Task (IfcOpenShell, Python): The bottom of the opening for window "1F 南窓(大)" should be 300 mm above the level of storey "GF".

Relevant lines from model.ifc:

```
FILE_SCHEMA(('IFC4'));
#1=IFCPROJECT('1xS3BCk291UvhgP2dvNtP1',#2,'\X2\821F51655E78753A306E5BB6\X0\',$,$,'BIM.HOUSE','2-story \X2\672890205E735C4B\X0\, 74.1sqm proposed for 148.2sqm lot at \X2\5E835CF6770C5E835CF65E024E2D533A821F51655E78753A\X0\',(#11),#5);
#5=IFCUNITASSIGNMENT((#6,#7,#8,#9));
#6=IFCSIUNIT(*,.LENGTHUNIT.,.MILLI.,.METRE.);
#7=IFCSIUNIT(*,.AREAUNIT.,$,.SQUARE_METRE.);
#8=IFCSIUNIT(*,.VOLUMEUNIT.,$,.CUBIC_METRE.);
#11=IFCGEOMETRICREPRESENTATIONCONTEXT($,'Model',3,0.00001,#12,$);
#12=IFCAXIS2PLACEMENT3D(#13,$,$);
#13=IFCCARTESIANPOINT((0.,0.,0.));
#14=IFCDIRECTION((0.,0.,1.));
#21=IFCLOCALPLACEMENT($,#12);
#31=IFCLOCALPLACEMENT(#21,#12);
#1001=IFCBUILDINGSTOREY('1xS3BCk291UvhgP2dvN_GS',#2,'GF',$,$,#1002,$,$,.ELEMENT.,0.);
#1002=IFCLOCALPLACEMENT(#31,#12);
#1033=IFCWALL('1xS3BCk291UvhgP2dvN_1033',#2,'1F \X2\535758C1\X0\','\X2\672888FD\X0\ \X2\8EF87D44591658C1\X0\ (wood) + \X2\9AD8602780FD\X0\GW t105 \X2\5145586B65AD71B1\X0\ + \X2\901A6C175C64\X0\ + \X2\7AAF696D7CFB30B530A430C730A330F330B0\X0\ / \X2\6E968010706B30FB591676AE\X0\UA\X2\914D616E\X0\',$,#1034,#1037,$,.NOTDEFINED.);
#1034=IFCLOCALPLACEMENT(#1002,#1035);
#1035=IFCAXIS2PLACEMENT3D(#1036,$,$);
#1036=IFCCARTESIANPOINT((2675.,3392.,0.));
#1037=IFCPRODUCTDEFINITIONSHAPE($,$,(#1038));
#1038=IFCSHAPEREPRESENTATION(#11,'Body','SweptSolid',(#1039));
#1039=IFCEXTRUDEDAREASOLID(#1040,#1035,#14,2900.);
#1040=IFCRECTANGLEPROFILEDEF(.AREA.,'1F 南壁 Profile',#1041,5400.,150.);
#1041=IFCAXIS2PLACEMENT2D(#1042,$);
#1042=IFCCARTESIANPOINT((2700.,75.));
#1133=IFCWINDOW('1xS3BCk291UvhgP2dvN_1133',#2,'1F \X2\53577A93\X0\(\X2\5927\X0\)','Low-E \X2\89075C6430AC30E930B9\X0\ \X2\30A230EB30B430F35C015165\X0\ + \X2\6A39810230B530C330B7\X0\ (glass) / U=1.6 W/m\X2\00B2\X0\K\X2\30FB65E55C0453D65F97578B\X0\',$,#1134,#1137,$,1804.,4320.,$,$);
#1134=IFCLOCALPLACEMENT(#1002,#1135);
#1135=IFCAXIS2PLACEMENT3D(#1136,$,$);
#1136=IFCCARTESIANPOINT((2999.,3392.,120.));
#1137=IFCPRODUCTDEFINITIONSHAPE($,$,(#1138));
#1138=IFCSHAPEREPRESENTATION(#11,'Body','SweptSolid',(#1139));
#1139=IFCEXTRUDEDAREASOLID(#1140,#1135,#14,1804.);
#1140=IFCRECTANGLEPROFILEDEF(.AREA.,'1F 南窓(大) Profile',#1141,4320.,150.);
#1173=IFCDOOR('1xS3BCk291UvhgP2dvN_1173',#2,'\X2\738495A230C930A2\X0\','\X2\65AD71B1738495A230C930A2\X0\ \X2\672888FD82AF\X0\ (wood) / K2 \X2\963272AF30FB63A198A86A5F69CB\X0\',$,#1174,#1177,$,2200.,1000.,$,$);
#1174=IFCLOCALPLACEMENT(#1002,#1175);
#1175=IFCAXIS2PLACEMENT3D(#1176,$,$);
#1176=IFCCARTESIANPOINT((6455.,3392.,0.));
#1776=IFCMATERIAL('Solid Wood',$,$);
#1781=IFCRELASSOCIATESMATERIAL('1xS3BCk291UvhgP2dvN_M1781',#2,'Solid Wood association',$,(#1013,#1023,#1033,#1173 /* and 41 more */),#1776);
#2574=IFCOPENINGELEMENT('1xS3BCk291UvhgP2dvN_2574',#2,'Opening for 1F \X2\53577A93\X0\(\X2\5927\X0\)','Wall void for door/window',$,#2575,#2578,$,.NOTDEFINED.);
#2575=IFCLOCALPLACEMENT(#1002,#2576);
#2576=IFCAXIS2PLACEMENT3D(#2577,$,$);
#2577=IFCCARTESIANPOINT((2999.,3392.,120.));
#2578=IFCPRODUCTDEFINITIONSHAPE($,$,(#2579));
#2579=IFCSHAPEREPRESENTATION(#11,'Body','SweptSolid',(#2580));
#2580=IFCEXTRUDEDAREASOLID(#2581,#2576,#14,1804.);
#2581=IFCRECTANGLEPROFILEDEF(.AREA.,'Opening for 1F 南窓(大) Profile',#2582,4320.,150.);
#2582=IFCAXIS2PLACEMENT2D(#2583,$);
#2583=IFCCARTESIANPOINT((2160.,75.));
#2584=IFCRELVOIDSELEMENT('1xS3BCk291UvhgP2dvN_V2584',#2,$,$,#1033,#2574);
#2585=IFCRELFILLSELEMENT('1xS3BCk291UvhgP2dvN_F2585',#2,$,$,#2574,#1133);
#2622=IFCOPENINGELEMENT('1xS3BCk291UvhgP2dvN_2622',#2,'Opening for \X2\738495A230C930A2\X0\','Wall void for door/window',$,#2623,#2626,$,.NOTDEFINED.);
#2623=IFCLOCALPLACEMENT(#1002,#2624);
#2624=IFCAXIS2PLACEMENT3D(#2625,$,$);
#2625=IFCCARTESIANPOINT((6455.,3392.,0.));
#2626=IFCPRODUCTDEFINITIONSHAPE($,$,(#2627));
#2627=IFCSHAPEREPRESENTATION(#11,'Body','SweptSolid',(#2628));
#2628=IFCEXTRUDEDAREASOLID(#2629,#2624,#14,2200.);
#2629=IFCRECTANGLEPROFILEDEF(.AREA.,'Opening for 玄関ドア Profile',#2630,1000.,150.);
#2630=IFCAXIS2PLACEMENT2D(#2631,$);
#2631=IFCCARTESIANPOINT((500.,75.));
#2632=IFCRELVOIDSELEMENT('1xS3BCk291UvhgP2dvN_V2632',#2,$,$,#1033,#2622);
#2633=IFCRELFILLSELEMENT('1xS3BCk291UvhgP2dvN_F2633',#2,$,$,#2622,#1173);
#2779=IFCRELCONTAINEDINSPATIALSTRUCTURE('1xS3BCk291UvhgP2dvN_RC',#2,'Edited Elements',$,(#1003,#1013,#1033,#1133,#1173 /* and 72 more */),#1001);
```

```python
import numpy as np
import ifcopenshell
import ifcopenshell.api.geometry
import ifcopenshell.geom
import ifcopenshell.util.element
import ifcopenshell.util.placement
import ifcopenshell.util.shape
import ifcopenshell.util.unit

model = ifcopenshell.open("model.ifc")
unit_scale = ifcopenshell.util.unit.calculate_unit_scale(model)

window = model.by_guid("1xS3BCk291UvhgP2dvN_1133")
opening = window.FillsVoids[0].RelatingOpeningElement
storey = ifcopenshell.util.element.get_container(window, ifc_class="IfcBuildingStorey")
level = ifcopenshell.util.placement.get_local_placement(storey.ObjectPlacement)[2, 3]

# The opening's origin need not be at the sill, so measure its lowest point.
shape = ifcopenshell.geom.create_shape(ifcopenshell.geom.settings(), opening)
bottom = ifcopenshell.util.shape.get_shape_bottom_elevation(shape, shape.geometry) / unit_scale
dz = level + 0.3 / unit_scale - bottom

shift = np.array([0.0, 0.0, dz])
# The window is not placed relative to its opening, so move both.
for product in (opening, window):
    matrix = ifcopenshell.util.placement.get_local_placement(product.ObjectPlacement)
    matrix[:3, 3] += shift
    ifcopenshell.api.geometry.edit_object_placement(model, product=product, matrix=matrix, is_si=False)

print(f"moved by {dz * unit_scale:+.3f} m")

model.write("model-out.ifc")
```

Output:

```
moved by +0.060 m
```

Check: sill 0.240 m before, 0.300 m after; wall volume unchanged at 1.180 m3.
